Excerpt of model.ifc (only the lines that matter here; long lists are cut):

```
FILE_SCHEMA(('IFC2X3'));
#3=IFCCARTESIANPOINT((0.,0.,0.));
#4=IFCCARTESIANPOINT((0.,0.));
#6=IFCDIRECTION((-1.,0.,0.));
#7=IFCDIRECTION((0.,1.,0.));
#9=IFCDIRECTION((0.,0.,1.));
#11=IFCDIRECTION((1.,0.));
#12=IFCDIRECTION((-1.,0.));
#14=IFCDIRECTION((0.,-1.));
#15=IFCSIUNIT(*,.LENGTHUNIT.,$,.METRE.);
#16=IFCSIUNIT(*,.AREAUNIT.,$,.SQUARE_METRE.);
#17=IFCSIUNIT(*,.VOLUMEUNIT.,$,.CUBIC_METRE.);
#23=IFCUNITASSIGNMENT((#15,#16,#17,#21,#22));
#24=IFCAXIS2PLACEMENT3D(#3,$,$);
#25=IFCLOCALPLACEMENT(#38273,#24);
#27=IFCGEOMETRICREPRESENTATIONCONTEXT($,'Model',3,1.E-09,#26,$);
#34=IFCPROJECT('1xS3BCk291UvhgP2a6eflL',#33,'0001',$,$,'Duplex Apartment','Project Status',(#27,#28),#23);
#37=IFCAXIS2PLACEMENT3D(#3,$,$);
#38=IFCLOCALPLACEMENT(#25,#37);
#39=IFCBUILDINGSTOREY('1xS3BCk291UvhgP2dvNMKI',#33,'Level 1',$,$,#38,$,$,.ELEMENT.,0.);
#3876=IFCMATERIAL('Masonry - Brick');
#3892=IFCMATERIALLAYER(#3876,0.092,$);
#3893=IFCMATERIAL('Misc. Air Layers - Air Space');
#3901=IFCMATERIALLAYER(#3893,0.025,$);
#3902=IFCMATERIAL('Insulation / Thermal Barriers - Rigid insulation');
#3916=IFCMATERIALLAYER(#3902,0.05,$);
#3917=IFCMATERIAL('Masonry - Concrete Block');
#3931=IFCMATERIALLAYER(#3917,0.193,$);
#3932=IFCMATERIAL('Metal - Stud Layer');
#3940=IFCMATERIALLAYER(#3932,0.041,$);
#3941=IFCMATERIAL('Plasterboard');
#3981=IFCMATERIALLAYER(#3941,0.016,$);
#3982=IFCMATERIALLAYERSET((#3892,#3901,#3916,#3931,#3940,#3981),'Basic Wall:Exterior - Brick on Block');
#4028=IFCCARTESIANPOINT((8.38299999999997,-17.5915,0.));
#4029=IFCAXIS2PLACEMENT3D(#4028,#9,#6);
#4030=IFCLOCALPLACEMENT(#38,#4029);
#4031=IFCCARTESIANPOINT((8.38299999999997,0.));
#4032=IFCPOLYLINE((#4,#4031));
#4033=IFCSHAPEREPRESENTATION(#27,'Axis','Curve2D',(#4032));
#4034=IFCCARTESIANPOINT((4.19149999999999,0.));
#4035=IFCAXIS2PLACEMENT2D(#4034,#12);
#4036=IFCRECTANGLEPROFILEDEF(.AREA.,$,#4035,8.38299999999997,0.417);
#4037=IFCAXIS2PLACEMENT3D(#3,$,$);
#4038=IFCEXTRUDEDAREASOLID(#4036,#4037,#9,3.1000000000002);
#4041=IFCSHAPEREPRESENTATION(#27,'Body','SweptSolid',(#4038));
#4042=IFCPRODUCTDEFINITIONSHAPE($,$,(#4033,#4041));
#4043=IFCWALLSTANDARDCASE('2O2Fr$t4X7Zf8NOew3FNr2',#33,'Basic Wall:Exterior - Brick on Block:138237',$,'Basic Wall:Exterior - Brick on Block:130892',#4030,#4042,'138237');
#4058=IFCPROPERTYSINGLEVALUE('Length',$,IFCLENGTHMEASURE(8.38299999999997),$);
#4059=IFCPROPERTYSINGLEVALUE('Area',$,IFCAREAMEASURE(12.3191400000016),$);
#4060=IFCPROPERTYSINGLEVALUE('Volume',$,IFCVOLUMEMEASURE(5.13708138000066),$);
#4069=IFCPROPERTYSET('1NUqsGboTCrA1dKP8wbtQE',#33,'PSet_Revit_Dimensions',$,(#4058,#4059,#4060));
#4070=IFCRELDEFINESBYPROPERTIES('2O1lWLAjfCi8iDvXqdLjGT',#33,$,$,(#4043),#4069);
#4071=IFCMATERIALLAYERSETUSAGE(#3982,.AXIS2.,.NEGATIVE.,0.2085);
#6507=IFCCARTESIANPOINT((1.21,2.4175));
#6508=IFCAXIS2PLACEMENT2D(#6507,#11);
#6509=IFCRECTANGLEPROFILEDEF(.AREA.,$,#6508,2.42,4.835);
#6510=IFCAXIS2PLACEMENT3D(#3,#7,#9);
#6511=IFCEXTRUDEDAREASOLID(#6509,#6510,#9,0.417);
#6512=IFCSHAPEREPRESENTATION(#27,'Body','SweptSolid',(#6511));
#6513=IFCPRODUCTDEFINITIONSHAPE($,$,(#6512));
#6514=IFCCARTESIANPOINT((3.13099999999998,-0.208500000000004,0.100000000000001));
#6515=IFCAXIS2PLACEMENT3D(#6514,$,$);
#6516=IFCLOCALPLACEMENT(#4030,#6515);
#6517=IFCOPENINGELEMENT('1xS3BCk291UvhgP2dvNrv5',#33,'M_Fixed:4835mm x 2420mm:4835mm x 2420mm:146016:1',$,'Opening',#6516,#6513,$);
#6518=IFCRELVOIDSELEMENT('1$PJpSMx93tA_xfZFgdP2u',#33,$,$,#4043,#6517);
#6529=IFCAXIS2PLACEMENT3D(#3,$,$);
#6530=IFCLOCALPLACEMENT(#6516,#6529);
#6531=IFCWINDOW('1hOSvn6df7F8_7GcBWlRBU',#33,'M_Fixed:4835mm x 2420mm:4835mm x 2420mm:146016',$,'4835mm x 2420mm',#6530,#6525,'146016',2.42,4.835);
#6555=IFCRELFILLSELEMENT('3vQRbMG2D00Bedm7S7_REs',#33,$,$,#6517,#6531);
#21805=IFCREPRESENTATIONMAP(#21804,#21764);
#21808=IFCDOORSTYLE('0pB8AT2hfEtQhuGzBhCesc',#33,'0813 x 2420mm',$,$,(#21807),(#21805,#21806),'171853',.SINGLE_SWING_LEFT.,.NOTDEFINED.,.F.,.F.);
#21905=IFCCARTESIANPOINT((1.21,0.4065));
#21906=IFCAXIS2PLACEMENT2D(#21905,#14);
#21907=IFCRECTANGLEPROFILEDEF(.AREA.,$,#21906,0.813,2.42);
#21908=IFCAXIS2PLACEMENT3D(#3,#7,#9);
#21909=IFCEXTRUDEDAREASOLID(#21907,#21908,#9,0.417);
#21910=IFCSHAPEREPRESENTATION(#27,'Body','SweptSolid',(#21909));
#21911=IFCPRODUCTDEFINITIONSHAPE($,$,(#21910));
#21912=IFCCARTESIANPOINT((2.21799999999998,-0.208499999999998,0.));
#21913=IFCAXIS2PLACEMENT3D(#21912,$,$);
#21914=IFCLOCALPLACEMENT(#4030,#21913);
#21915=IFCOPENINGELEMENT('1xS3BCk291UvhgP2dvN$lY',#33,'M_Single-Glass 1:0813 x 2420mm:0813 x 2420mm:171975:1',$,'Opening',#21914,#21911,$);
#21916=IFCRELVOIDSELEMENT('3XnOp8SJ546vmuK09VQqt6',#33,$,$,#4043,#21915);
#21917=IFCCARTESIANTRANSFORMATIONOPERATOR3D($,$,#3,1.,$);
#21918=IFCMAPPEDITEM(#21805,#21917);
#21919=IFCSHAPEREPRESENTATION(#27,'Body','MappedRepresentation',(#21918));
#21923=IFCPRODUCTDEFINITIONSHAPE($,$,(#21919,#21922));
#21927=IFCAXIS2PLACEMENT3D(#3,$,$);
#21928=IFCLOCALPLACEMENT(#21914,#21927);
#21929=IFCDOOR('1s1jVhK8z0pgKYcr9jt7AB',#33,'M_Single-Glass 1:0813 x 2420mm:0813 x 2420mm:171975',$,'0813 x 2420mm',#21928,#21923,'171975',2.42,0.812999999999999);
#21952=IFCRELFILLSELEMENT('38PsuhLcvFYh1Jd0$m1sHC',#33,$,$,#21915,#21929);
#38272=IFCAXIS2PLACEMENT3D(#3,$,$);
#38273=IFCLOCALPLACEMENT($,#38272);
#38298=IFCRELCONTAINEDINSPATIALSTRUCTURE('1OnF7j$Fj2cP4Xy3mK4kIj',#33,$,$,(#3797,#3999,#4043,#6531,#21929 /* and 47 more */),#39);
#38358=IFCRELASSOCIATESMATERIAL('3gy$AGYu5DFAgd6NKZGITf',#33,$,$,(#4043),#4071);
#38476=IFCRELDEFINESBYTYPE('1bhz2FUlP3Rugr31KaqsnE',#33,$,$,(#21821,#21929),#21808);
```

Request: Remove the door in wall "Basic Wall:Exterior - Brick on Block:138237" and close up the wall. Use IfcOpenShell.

```python
import ifcopenshell
import ifcopenshell.api.feature
import ifcopenshell.api.pset
import ifcopenshell.api.root
import ifcopenshell.geom
import ifcopenshell.util.element
import ifcopenshell.util.shape
import ifcopenshell.util.unit

model = ifcopenshell.open("model.ifc")
area_scale = ifcopenshell.util.unit.calculate_unit_scale(model, "AREAUNIT")
volume_scale = ifcopenshell.util.unit.calculate_unit_scale(model, "VOLUMEUNIT")
settings = ifcopenshell.geom.settings()


def volume(element):
    """Net volume in cubic metres, openings subtracted."""
    shape = ifcopenshell.geom.create_shape(settings, element)
    return ifcopenshell.util.shape.get_volume(shape.geometry)


door = model.by_guid("1s1jVhK8z0pgKYcr9jt7AB")
opening = door.FillsVoids[0].RelatingOpeningElement
wall = opening.VoidsElements[0].RelatingBuildingElement
before = volume(wall)

ifcopenshell.api.root.remove_product(model, product=door)
ifcopenshell.api.feature.remove_feature(model, feature=opening)

after = volume(wall)
thickness = 0.417  # wall thickness in metres

# Update the wall's stored quantities.
pset = model.by_id(ifcopenshell.util.element.get_pset(wall, "PSet_Revit_Dimensions", should_inherit=False)["id"])
ifcopenshell.api.pset.edit_pset(model, pset=pset, properties={
    "Area": model.create_entity("IfcAreaMeasure", after / thickness / area_scale),
    "Volume": model.create_entity("IfcVolumeMeasure", after / volume_scale),
})

print(f"wall volume {before:.3f} -> {after:.3f} m3")

model.write("model_updated.ifc")
```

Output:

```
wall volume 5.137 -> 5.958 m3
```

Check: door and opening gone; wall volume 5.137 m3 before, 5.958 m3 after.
